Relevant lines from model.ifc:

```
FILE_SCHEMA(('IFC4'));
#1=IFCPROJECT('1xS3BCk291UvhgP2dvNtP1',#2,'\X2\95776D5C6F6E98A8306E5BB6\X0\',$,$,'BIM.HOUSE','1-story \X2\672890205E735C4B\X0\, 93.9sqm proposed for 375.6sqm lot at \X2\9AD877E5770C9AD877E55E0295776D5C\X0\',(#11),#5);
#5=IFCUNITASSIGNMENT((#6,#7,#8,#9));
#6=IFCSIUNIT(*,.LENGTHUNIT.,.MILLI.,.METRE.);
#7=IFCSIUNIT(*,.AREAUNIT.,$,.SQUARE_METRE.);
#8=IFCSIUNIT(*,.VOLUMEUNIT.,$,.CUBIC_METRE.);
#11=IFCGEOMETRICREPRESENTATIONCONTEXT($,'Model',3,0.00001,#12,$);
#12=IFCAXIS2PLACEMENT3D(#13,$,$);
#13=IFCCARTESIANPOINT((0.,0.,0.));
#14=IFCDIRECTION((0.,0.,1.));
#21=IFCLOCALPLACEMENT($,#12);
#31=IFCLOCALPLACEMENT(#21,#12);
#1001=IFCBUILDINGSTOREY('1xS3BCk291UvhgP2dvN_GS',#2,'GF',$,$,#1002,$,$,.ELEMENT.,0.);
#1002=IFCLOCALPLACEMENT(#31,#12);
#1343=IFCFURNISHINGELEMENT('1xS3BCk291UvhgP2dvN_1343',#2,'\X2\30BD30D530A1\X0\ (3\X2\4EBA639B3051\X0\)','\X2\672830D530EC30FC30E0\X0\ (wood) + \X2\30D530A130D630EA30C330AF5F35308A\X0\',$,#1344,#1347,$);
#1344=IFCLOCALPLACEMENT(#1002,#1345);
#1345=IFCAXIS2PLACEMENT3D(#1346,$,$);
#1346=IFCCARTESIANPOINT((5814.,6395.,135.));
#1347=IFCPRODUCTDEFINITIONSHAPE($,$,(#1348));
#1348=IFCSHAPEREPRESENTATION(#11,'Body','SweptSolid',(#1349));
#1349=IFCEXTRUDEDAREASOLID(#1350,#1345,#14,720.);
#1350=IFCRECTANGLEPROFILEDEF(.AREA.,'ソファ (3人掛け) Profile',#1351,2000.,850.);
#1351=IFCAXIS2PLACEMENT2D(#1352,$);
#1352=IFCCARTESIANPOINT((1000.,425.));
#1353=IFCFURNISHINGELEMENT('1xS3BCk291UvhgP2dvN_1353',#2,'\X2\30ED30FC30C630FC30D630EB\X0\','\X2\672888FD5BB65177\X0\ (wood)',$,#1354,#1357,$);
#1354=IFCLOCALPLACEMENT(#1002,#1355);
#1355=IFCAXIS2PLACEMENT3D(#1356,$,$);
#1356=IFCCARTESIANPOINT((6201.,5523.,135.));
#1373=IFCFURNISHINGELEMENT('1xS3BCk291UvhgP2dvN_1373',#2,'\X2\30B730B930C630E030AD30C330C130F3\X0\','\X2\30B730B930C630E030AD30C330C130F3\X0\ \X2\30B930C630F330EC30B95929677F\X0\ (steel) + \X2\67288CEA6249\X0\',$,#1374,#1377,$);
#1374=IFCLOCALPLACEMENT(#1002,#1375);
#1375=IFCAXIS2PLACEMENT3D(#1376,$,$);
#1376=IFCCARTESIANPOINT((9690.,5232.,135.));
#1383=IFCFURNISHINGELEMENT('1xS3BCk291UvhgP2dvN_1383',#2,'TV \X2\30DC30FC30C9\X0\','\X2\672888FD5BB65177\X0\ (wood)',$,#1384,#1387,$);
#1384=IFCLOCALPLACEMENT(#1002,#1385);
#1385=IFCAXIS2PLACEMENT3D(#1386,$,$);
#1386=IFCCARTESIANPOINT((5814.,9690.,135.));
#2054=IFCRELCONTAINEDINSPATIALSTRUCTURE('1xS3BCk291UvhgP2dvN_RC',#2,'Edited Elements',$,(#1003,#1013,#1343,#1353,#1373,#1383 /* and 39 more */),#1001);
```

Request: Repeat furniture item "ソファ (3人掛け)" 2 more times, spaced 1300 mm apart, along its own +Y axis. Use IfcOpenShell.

```python
import ifcopenshell
import ifcopenshell.api.geometry
import ifcopenshell.api.root
import ifcopenshell.util.element
import ifcopenshell.util.placement
import ifcopenshell.util.unit

model = ifcopenshell.open("model.ifc")
unit_scale = ifcopenshell.util.unit.calculate_unit_scale(model)


def reuse_history(source, copy):
    """copy_class also copies each property set's owner history, people and application; keep the originals."""
    for rel in copy.IsDefinedBy:
        if rel.is_a("IfcRelDefinesByProperties") and (history := rel.RelatingPropertyDefinition.OwnerHistory):
            rel.RelatingPropertyDefinition.OwnerHistory = source.OwnerHistory
            ifcopenshell.util.element.remove_deep2(model, history)


source = model.by_id(1343)
base = ifcopenshell.util.placement.get_local_placement(source.ObjectPlacement)
step = base[:3, 1] * 1.3 / unit_scale

for i in range(1, 3):
    copy = ifcopenshell.api.root.copy_class(model, product=source)
    copy.Representation = ifcopenshell.util.element.copy_deep(
        model, source.Representation, exclude=["IfcGeometricRepresentationContext", "IfcRepresentationMap"]
    )
    reuse_history(source, copy)
    matrix = base.copy()
    matrix[:3, 3] += i * step
    print("added at", matrix[:3, 3].round(3) + 0.0)
    ifcopenshell.api.geometry.edit_object_placement(model, product=copy, matrix=matrix, is_si=False)

model.write("model_v2.ifc")
```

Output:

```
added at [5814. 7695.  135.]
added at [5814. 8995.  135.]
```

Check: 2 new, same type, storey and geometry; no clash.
